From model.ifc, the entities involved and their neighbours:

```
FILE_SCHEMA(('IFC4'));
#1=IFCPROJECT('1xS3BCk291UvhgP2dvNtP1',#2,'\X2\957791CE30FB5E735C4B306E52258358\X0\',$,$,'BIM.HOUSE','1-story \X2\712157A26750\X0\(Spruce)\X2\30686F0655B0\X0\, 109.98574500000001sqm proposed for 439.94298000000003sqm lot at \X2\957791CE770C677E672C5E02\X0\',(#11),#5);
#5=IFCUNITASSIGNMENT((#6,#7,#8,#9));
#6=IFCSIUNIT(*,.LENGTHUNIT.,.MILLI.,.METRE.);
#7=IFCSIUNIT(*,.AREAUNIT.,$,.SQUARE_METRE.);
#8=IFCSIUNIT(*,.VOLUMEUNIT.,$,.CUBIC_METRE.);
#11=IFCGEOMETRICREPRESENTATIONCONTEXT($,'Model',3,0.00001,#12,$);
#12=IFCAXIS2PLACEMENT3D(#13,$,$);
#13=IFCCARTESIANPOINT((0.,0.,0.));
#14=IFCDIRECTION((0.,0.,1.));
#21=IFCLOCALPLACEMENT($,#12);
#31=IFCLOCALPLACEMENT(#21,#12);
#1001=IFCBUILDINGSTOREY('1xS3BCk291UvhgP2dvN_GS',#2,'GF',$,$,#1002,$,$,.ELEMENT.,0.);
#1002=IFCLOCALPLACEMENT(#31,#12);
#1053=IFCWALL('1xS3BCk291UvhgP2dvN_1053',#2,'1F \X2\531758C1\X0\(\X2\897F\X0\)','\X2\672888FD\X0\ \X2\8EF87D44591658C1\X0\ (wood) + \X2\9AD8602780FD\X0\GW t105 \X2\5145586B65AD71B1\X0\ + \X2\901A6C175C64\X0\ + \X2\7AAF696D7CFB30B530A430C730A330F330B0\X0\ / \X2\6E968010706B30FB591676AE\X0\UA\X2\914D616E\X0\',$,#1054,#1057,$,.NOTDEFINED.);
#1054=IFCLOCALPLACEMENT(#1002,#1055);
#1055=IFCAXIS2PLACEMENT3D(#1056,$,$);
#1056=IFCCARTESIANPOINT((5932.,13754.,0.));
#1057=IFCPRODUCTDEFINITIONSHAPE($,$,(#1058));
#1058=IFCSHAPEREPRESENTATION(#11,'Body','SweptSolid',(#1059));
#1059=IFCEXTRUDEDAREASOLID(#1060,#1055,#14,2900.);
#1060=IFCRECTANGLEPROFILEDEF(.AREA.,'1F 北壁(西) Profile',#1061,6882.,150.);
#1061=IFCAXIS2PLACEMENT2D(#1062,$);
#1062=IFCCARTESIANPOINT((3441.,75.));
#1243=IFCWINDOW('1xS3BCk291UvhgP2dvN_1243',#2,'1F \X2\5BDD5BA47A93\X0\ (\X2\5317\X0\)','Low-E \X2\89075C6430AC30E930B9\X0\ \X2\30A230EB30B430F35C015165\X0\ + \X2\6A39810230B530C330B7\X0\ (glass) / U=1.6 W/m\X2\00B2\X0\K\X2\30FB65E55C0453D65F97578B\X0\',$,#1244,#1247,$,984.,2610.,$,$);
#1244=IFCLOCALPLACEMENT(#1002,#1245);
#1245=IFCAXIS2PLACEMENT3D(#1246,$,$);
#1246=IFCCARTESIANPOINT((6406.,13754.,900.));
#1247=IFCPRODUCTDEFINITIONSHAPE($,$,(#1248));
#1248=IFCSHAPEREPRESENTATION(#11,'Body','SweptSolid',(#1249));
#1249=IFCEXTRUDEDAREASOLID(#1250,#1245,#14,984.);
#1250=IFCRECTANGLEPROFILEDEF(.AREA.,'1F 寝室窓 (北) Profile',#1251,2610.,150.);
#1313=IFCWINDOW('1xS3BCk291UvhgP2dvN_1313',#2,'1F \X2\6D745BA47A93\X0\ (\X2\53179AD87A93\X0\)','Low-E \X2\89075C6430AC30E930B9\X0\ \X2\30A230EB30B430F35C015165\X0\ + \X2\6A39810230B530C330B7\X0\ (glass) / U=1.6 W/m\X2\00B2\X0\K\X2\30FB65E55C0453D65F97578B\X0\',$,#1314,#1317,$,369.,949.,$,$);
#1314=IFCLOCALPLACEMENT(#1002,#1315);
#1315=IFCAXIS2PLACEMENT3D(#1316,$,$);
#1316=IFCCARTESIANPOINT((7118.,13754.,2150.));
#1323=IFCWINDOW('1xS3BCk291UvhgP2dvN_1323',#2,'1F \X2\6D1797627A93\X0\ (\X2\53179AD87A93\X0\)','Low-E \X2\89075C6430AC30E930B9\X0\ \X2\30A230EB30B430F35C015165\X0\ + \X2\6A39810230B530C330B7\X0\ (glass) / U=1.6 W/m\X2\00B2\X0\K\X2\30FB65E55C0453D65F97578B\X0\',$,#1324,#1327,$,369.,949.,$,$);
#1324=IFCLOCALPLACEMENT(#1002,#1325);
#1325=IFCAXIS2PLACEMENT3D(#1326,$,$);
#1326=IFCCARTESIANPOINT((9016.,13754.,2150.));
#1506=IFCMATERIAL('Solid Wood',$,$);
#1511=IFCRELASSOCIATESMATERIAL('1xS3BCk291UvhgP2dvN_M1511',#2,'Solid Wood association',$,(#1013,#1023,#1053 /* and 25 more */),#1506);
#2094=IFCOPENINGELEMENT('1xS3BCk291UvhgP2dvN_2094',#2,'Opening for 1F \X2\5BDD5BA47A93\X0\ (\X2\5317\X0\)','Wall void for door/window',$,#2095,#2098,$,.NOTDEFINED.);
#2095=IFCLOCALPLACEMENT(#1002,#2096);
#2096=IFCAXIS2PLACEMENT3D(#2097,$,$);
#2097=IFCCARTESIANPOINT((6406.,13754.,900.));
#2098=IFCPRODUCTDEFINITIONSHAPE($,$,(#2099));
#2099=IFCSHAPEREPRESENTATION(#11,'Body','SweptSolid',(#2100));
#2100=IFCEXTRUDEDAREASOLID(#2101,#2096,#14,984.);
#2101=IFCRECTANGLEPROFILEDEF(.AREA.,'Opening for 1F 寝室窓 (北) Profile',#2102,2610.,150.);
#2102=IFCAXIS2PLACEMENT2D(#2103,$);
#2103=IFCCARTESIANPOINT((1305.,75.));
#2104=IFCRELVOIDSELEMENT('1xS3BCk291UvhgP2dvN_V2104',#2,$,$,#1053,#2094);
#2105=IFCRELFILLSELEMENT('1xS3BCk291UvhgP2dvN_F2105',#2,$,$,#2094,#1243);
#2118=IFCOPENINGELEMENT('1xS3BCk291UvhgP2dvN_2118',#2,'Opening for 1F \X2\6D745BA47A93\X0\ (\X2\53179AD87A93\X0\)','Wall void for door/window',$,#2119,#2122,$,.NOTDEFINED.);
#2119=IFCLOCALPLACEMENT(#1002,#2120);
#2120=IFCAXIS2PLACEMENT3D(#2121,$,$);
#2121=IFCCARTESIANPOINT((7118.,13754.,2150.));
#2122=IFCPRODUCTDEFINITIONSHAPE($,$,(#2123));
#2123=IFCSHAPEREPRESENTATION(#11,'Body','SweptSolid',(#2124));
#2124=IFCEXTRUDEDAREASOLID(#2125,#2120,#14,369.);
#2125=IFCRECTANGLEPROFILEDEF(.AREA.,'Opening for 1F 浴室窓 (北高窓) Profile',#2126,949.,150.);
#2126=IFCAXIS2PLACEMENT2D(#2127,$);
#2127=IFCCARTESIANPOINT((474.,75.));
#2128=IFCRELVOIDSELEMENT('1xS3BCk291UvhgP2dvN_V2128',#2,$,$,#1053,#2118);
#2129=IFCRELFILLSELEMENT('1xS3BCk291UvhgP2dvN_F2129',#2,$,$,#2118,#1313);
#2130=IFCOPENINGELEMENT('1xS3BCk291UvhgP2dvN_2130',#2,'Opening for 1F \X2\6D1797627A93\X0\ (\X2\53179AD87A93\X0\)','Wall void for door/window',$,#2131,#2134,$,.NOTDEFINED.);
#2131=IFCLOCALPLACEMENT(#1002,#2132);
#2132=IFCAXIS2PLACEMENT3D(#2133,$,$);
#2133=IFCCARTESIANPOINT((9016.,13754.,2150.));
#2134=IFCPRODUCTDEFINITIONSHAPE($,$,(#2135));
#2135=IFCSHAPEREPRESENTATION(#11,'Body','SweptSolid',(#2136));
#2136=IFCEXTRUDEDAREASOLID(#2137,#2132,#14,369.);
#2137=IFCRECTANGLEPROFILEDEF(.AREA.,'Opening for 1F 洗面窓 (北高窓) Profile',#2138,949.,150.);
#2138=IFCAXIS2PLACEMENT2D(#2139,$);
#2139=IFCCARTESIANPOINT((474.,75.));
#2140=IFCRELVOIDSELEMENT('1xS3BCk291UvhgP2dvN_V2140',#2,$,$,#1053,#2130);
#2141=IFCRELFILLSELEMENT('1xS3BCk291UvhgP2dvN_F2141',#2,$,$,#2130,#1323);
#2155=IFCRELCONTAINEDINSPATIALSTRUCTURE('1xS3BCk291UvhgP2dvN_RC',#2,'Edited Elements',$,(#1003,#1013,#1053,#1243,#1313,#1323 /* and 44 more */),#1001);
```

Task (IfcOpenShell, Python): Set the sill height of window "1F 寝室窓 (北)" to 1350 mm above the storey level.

```python
import numpy as np
import ifcopenshell
import ifcopenshell.api.geometry
import ifcopenshell.geom
import ifcopenshell.util.element
import ifcopenshell.util.placement
import ifcopenshell.util.shape
import ifcopenshell.util.unit

model = ifcopenshell.open("model.ifc")
unit_scale = ifcopenshell.util.unit.calculate_unit_scale(model)

window = model.by_guid("1xS3BCk291UvhgP2dvN_1243")
opening = window.FillsVoids[0].RelatingOpeningElement
storey = ifcopenshell.util.element.get_container(window, ifc_class="IfcBuildingStorey")
level = ifcopenshell.util.placement.get_local_placement(storey.ObjectPlacement)[2, 3]

# The opening's origin need not be at the sill, so measure its lowest point.
shape = ifcopenshell.geom.create_shape(ifcopenshell.geom.settings(), opening)
bottom = ifcopenshell.util.shape.get_shape_bottom_elevation(shape, shape.geometry) / unit_scale
dz = level + 1.35 / unit_scale - bottom

shift = np.array([0.0, 0.0, dz])
# The window is not placed relative to its opening, so move both.
for product in (opening, window):
    matrix = ifcopenshell.util.placement.get_local_placement(product.ObjectPlacement)
    matrix[:3, 3] += shift
    ifcopenshell.api.geometry.edit_object_placement(model, product=product, matrix=matrix, is_si=False)

print(f"moved by {dz * unit_scale:+.3f} m")

model.write("model_updated.ifc")
```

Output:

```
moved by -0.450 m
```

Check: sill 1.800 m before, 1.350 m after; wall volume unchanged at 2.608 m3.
